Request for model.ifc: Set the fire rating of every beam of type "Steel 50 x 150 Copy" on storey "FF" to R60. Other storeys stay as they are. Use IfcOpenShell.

First a look at what the model holds.

```python
import ifcopenshell
import ifcopenshell.util.element

model = ifcopenshell.open("model.ifc")
print(model.schema)
storey = next(s for s in model.by_type("IfcBuildingStorey") if s.Name == "FF")
beams = [e for e in ifcopenshell.util.element.get_decomposition(storey) if e.is_a("IfcBeam")]
seen = {}
for e in beams:
    element_type = ifcopenshell.util.element.get_type(e)
    key = (element_type.Name if element_type != e and element_type else None, ifcopenshell.util.element.get_pset(e, "Pset_BeamCommon", "FireRating"))
    seen[key] = seen.get(key, 0) + 1
for (name, value), count in sorted(seen.items(), key=str):
    print(count, "x", name, "|", value)
```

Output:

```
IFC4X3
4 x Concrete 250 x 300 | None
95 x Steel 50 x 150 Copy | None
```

```python
import ifcopenshell
import ifcopenshell.api.pset
import ifcopenshell.util.element

model = ifcopenshell.open("model.ifc")

storey = next(s for s in model.by_type("IfcBuildingStorey") if s.Name == "FF")
beams = [e for e in ifcopenshell.util.element.get_decomposition(storey) if e.is_a("IfcBeam")]

count = 0
for e in beams:
    element_type = ifcopenshell.util.element.get_type(e)
    if element_type in (None, e) or element_type.Name != "Steel 50 x 150 Copy":
        continue
    # add_pset returns the element's existing set when there is one.
    pset = ifcopenshell.api.pset.add_pset(model, product=e, name="Pset_BeamCommon")
    ifcopenshell.api.pset.edit_pset(model, pset=pset, properties={"FireRating": "R60"})
    count += 1

print(count, "beams updated")

model.write("model-out.ifc")
```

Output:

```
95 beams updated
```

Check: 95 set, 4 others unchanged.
